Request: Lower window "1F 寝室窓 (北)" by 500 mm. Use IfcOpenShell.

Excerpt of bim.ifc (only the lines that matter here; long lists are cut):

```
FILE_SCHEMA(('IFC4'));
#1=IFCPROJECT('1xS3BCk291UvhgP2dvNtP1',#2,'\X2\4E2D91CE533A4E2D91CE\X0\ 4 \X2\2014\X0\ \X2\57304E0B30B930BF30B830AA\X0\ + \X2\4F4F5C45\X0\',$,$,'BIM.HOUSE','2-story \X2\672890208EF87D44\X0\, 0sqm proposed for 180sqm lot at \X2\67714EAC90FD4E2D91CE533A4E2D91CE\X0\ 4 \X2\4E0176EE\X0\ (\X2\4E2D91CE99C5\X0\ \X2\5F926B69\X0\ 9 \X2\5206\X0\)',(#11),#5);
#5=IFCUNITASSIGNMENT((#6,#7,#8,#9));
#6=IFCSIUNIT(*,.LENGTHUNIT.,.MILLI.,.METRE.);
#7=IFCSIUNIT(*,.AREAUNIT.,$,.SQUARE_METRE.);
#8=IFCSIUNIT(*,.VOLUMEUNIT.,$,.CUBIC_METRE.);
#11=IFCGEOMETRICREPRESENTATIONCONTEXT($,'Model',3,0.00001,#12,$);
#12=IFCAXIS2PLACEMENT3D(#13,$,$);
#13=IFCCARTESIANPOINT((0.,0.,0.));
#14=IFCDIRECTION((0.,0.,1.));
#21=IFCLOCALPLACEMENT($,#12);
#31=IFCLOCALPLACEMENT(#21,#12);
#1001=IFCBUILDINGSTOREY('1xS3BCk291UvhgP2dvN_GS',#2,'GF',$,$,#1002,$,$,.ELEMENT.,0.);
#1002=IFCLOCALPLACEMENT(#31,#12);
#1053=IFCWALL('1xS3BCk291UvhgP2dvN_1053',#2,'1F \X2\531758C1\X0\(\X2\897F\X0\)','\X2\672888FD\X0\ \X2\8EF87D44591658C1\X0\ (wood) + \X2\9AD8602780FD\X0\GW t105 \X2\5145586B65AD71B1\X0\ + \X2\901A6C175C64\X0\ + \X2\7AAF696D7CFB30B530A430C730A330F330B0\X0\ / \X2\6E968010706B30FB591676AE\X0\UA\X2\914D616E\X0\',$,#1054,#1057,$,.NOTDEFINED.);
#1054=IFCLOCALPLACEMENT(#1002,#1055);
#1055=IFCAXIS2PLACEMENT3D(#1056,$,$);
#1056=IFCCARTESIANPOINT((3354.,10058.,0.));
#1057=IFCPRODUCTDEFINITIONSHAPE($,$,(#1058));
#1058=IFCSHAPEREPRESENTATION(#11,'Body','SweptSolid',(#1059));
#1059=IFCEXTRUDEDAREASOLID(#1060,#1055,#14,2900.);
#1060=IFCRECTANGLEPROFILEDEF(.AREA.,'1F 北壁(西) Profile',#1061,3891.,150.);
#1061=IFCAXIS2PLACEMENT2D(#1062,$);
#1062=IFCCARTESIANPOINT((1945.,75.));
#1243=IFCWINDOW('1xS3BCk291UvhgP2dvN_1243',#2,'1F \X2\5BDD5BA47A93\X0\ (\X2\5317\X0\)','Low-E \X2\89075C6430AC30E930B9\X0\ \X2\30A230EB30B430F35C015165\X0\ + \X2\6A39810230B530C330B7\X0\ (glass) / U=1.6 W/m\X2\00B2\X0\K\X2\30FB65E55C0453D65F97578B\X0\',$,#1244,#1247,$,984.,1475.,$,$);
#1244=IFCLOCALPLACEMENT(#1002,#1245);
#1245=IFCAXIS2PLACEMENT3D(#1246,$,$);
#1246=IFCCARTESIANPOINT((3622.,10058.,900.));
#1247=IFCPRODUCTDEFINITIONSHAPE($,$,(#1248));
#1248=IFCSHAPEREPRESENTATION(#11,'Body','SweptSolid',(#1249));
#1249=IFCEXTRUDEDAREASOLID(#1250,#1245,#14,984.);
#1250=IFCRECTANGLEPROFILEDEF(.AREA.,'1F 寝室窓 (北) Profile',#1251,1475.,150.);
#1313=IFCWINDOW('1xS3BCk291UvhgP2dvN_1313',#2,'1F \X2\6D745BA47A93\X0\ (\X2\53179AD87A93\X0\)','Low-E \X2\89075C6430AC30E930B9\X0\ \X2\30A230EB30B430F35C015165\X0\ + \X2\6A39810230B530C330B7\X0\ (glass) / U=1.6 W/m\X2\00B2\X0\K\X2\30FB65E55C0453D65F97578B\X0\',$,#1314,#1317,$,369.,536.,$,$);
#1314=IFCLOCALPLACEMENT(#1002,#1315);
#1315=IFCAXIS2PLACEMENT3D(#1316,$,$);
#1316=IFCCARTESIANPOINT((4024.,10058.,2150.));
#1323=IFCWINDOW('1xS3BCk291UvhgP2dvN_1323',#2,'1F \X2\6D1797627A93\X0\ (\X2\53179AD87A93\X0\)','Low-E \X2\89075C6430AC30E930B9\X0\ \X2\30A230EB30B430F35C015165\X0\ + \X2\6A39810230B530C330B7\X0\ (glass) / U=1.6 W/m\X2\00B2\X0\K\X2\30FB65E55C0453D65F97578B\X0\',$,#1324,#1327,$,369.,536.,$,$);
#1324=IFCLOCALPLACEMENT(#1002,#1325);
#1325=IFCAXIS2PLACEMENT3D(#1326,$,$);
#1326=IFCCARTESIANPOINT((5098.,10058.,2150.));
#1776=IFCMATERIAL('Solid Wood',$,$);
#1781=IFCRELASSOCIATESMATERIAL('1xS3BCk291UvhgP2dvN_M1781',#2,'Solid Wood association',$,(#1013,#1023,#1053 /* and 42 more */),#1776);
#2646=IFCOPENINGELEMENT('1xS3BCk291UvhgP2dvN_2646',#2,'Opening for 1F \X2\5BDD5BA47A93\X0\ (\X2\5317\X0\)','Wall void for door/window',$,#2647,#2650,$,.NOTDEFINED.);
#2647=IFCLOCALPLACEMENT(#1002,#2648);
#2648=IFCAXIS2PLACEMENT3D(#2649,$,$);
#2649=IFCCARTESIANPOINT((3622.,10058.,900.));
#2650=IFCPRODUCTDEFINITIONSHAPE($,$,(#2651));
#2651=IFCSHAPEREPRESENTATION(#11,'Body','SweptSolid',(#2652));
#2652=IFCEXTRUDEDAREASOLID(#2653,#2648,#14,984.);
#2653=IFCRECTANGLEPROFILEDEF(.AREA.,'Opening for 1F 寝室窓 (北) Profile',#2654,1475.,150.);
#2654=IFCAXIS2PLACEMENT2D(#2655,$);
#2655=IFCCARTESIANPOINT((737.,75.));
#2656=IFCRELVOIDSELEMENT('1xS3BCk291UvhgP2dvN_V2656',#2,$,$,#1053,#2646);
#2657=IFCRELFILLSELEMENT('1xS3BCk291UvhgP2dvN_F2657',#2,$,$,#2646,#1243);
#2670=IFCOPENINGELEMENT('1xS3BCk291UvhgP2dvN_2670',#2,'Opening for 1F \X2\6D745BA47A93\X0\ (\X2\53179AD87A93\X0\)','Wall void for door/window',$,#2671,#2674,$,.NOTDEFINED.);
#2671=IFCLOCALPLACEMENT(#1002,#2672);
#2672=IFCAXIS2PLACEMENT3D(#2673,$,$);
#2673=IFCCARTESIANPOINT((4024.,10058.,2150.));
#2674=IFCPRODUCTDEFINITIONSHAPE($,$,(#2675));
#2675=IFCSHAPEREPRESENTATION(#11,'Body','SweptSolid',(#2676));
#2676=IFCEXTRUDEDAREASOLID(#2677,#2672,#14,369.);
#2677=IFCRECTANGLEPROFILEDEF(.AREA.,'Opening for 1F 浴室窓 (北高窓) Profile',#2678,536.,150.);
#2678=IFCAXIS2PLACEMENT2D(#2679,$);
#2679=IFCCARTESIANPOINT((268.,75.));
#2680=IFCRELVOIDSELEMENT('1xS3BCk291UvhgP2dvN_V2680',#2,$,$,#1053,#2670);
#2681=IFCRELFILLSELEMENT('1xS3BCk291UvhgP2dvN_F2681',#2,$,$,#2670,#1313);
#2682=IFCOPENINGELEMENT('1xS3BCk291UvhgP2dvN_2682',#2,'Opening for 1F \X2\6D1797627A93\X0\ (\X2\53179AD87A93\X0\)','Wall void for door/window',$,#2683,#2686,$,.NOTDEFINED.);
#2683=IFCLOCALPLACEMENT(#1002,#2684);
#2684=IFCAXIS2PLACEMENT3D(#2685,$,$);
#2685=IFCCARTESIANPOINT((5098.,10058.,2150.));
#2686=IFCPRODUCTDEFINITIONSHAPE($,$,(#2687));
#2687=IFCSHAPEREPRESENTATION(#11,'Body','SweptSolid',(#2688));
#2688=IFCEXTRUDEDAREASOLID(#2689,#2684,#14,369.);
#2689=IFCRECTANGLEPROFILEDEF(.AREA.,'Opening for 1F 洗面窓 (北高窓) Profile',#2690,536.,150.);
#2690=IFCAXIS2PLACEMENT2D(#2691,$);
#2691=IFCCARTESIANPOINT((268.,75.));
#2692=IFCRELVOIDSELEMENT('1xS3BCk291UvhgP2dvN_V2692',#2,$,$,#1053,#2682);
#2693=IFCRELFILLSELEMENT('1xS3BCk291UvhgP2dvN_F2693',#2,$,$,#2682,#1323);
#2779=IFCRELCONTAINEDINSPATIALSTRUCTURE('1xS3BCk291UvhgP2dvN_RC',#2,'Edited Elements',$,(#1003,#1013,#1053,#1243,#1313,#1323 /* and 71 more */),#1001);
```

```python
import numpy as np
import ifcopenshell
import ifcopenshell.api.geometry
import ifcopenshell.util.placement
import ifcopenshell.util.unit

model = ifcopenshell.open("bim.ifc")
unit_scale = ifcopenshell.util.unit.calculate_unit_scale(model)

window = model.by_id(1243)
opening = window.FillsVoids[0].RelatingOpeningElement
dz = -0.5 / unit_scale

shift = np.array([0.0, 0.0, dz])
# The window is not placed relative to its opening, so move both.
for product in (opening, window):
    matrix = ifcopenshell.util.placement.get_local_placement(product.ObjectPlacement)
    matrix[:3, 3] += shift
    ifcopenshell.api.geometry.edit_object_placement(model, product=product, matrix=matrix, is_si=False)

print(f"moved by {dz * unit_scale:+.3f} m")

model.write("bim_edited.ifc")
```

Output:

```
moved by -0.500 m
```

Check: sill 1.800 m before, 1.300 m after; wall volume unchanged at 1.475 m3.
